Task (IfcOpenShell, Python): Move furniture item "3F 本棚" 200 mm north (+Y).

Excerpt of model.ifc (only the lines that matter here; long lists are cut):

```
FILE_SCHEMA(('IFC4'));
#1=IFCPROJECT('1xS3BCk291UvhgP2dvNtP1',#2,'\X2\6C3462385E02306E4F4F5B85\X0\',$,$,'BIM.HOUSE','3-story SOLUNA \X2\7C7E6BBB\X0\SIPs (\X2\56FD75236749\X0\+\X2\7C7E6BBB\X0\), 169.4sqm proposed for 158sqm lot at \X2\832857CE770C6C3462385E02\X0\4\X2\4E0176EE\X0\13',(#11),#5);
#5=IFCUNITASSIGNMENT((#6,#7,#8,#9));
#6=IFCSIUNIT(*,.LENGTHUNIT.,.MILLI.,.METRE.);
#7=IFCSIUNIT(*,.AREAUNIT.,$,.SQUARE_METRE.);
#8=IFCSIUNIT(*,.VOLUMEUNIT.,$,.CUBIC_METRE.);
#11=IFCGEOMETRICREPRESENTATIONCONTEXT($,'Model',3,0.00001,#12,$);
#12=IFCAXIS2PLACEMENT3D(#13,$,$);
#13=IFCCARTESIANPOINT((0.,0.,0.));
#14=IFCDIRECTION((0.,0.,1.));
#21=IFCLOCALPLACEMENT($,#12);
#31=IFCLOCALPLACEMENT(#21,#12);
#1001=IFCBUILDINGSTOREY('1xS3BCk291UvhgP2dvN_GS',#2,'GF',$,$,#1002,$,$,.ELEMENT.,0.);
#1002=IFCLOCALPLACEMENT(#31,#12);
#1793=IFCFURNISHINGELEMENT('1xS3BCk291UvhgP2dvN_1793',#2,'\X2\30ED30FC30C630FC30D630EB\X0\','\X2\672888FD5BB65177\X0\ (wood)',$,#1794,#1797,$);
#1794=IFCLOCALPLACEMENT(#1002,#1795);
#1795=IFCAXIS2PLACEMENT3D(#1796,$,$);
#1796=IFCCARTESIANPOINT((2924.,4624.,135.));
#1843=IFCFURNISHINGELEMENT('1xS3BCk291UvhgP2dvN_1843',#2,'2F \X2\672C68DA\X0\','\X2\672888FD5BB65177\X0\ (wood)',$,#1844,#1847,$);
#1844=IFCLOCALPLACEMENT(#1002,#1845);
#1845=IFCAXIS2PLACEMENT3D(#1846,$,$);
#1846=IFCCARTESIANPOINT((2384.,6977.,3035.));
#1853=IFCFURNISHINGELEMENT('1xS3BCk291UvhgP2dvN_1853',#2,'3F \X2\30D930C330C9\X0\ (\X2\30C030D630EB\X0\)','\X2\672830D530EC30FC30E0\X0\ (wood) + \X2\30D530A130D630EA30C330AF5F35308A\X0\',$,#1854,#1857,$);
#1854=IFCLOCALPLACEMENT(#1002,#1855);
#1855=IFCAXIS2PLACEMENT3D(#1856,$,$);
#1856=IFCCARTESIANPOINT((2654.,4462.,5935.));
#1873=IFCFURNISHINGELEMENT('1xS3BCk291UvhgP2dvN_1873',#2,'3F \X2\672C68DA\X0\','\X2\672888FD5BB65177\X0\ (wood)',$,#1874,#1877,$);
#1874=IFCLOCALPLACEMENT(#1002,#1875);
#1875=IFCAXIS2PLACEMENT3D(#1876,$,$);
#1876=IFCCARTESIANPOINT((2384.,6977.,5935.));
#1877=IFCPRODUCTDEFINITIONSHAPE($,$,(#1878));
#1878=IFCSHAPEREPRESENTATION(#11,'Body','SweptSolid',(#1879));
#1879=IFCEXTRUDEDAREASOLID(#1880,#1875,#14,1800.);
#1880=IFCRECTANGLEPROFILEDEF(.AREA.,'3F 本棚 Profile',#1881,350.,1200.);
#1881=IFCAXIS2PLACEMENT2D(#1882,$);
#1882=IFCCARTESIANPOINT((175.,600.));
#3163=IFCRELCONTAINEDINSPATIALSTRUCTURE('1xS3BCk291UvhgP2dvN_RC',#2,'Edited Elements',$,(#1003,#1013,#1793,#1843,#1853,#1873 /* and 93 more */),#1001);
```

```python
import ifcopenshell
import ifcopenshell.api.geometry
import ifcopenshell.util.placement
import ifcopenshell.util.unit

model = ifcopenshell.open("model.ifc")
unit_scale = ifcopenshell.util.unit.calculate_unit_scale(model)

item = model.by_id(1873)
matrix = ifcopenshell.util.placement.get_local_placement(item.ObjectPlacement)
matrix[1, 3] += 0.2 / unit_scale
ifcopenshell.api.geometry.edit_object_placement(model, product=item, matrix=matrix, is_si=False)

print(ifcopenshell.util.placement.get_local_placement(item.ObjectPlacement).round(3) + 0.0)

model.write("model_rev.ifc")
```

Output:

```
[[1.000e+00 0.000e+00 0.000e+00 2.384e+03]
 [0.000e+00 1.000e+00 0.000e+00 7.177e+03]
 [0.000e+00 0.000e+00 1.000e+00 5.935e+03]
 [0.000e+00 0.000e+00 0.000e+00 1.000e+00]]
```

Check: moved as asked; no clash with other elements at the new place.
